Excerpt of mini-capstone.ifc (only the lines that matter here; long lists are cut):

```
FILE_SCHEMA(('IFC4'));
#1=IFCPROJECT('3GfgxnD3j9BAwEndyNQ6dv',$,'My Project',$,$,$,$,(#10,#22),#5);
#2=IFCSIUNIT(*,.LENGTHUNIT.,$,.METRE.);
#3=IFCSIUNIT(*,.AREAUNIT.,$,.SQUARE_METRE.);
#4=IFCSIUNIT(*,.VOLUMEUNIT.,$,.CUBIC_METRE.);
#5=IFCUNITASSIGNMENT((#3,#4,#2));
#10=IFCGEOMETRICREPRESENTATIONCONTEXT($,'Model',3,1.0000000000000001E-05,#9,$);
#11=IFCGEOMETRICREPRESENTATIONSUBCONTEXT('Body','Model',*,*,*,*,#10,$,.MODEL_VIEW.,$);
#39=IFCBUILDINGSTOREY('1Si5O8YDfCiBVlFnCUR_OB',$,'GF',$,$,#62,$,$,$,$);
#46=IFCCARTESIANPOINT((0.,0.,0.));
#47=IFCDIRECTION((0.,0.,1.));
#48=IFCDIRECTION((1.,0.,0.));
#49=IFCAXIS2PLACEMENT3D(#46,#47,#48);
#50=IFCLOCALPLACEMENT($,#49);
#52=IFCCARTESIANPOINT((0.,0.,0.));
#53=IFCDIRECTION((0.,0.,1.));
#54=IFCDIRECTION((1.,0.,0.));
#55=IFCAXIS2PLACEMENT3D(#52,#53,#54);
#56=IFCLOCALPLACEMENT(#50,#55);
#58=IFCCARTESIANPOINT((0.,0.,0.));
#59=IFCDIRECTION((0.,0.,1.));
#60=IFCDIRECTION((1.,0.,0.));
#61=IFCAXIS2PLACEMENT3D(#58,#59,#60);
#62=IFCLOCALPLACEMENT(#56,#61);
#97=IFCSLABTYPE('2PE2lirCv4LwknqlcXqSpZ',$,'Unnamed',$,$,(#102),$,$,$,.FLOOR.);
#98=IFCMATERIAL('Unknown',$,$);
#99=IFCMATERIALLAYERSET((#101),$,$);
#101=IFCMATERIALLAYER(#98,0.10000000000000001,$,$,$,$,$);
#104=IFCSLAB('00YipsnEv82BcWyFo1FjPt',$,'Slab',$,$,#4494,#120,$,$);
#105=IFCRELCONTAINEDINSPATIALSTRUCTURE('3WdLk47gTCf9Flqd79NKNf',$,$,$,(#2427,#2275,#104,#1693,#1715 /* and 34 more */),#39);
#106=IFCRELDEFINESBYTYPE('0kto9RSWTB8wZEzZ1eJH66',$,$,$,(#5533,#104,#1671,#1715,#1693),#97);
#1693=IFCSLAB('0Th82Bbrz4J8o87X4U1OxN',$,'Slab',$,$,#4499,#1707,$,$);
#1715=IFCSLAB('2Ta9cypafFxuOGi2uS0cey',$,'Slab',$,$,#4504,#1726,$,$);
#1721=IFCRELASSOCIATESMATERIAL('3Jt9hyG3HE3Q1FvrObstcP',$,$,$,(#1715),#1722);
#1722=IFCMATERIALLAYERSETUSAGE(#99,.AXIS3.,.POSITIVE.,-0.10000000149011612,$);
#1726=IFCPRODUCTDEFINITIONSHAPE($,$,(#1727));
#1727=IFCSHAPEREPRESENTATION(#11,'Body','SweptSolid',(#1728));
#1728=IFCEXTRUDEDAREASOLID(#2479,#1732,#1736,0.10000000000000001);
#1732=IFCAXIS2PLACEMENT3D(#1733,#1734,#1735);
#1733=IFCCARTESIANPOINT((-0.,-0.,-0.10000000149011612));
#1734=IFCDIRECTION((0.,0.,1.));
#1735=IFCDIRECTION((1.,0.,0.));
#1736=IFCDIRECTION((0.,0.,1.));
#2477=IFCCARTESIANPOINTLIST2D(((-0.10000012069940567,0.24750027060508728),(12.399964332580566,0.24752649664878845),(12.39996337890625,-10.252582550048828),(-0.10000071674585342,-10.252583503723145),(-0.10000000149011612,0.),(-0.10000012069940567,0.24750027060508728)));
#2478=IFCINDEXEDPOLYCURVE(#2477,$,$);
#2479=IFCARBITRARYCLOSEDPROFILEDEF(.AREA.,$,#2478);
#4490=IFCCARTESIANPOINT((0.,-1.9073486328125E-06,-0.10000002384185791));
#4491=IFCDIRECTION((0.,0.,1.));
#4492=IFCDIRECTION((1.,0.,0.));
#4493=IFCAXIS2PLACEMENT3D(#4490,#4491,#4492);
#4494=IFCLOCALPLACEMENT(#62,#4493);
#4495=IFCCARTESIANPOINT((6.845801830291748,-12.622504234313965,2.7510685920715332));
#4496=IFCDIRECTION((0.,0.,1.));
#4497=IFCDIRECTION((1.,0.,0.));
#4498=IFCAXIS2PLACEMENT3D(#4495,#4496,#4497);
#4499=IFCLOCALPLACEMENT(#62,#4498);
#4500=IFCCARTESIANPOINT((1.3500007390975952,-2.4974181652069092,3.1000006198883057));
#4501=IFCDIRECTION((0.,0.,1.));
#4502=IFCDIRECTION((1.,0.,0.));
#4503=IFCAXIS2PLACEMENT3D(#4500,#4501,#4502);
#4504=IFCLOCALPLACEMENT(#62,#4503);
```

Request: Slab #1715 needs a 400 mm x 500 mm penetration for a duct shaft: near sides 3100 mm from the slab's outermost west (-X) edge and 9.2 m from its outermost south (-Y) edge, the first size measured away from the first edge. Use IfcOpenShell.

```python
import numpy as np
import ifcopenshell
import ifcopenshell.api.feature
import ifcopenshell.api.geometry
import ifcopenshell.api.root
import ifcopenshell.geom
import ifcopenshell.util.placement
import ifcopenshell.util.representation
import ifcopenshell.util.shape
import ifcopenshell.util.unit

model = ifcopenshell.open("mini-capstone.ifc")
unit_scale = ifcopenshell.util.unit.calculate_unit_scale(model)
settings = ifcopenshell.geom.settings()


def volume(element):
    """Net volume in cubic metres, openings subtracted."""
    shape = ifcopenshell.geom.create_shape(settings, element)
    return ifcopenshell.util.shape.get_volume(shape.geometry)


slab = model.by_id(1715)
before = volume(slab)

# Extent in the slab's own axes, in metres. The edges named are its -X and -Y sides.
slab_shape = ifcopenshell.geom.create_shape(settings, slab)
vertices = ifcopenshell.util.shape.get_vertices(slab_shape.geometry)
x_min, y_min, bottom = vertices.min(axis=0)
top = vertices[:, 2].max()

opening = ifcopenshell.api.root.create_entity(model, ifc_class="IfcOpeningElement", name="Duct shaft opening", predefined_type="OPENING")
context = ifcopenshell.util.representation.get_context(model, "Model", "Body", "MODEL_VIEW")
width, depth = 0.4, 0.5
outline = [(0.0, 0.0), (width, 0.0), (width, depth), (0.0, depth), (0.0, 0.0)]
# Overshoot both faces by 50 mm so the cut is clean.
shape = ifcopenshell.api.geometry.add_slab_representation(
    model, context=context, depth=top - bottom + 0.1, polyline=outline
)
ifcopenshell.api.geometry.assign_representation(model, product=opening, representation=shape)

matrix = ifcopenshell.util.placement.get_local_placement(slab.ObjectPlacement)
matrix[:, 3] = matrix @ np.append(np.array([x_min + 3.1, y_min + 9.2, bottom - 0.05]) / unit_scale, 1.0)
ifcopenshell.api.geometry.edit_object_placement(model, product=opening, matrix=matrix, is_si=False)
ifcopenshell.api.feature.add_feature(model, feature=opening, element=slab)

after = volume(slab)

print(f"slab volume {before:.3f} -> {after:.3f} m3")

model.write("mini-capstone_updated.ifc")
```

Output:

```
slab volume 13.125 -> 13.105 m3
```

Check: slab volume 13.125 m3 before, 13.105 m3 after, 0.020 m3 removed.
